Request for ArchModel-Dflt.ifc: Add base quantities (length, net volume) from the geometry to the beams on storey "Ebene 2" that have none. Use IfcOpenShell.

First a look at what the model holds.

```python
import ifcopenshell
import ifcopenshell.util.element
import ifcopenshell.util.unit

model = ifcopenshell.open("ArchModel-Dflt.ifc")
print(model.schema)
for unit_type in ("LENGTHUNIT", "AREAUNIT", "VOLUMEUNIT"):
    print(unit_type, ifcopenshell.util.unit.calculate_unit_scale(model, unit_type))
storey = next(s for s in model.by_type("IfcBuildingStorey") if s.Name == "Ebene 2")
beams = [e for e in ifcopenshell.util.element.get_decomposition(storey) if e.is_a("IfcBeam")]
for e in sorted(beams, key=lambda e: e.id()):
    print(e.id(), e.is_a(), e.Name, list(ifcopenshell.util.element.get_psets(e, qtos_only=True)), sep=" | ")
```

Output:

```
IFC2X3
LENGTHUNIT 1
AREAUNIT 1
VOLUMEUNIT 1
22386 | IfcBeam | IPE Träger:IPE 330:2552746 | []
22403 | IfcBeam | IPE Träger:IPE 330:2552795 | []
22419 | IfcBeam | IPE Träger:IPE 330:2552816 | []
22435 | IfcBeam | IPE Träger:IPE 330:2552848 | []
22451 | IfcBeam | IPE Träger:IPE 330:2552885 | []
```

```python
import ifcopenshell
import ifcopenshell.api.pset
import ifcopenshell.geom
import ifcopenshell.util.element
import ifcopenshell.util.shape
import ifcopenshell.util.unit

model = ifcopenshell.open("ArchModel-Dflt.ifc")
unit_scale = ifcopenshell.util.unit.calculate_unit_scale(model)
volume_scale = ifcopenshell.util.unit.calculate_unit_scale(model, "VOLUMEUNIT")
settings = ifcopenshell.geom.settings()

storey = next(s for s in model.by_type("IfcBuildingStorey") if s.Name == "Ebene 2")
beams = [e for e in ifcopenshell.util.element.get_decomposition(storey) if e.is_a("IfcBeam")]

for e in sorted(beams, key=lambda e: e.id()):
    if ifcopenshell.util.element.get_psets(e, qtos_only=True, should_inherit=False):
        continue
    # Geometry comes back in metres, in the element's own axes.
    shape = ifcopenshell.geom.create_shape(settings, e)
    values = {
        "Length": ifcopenshell.util.shape.get_max_xyz(shape.geometry) / unit_scale,
        "NetVolume": ifcopenshell.util.shape.get_volume(shape.geometry) / volume_scale,
    }
    qto = ifcopenshell.api.pset.add_qto(model, product=e, name="BaseQuantities")
    ifcopenshell.api.pset.edit_qto(model, qto=qto, properties=values)
    print(e.id(), {k: round(v, 3) for k, v in values.items()})

model.write("ArchModel-Dflt_edited.ifc")
```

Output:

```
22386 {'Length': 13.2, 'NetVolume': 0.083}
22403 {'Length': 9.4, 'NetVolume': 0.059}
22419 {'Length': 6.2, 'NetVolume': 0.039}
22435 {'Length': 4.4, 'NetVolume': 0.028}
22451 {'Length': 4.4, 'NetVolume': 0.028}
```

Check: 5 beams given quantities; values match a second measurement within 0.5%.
